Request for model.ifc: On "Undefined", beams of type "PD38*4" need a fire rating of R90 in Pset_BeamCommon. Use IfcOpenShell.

First a look at what the model holds.

```python
import ifcopenshell
import ifcopenshell.util.element

model = ifcopenshell.open("model.ifc")
print(model.schema)
storey = next(s for s in model.by_type("IfcBuildingStorey") if s.Name == "Undefined")
beams = [e for e in ifcopenshell.util.element.get_decomposition(storey) if e.is_a("IfcBeam")]
seen = {}
for e in beams:
    element_type = ifcopenshell.util.element.get_type(e)
    key = (element_type.Name if element_type != e and element_type else None, ifcopenshell.util.element.get_pset(e, "Pset_BeamCommon", "FireRating"))
    seen[key] = seen.get(key, 0) + 1
for (name, value), count in sorted(seen.items(), key=str):
    print(count, "x", name, "|", value)
```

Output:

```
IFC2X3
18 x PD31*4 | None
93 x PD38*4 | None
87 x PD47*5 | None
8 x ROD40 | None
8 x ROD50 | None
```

```python
import ifcopenshell
import ifcopenshell.api.pset
import ifcopenshell.util.element

model = ifcopenshell.open("model.ifc")

storey = next(s for s in model.by_type("IfcBuildingStorey") if s.Name == "Undefined")
beams = [e for e in ifcopenshell.util.element.get_decomposition(storey) if e.is_a("IfcBeam")]

count = 0
for e in beams:
    element_type = ifcopenshell.util.element.get_type(e)
    if element_type in (None, e) or element_type.Name != "PD38*4":
        continue
    found = ifcopenshell.util.element.get_pset(e, "Pset_BeamCommon", should_inherit=False)
    if found:
        pset = model.by_id(found["id"])
        if len(ifcopenshell.util.element.get_elements_by_pset(pset)) > 1:
            pset = ifcopenshell.api.pset.unshare_pset(model, products=[e], pset=pset)[0]
    else:
        pset = ifcopenshell.api.pset.add_pset(model, product=e, name="Pset_BeamCommon")
    ifcopenshell.api.pset.edit_pset(model, pset=pset, properties={"FireRating": "R90"})
    count += 1

print(count, "beams updated")

model.write("model-out.ifc")
```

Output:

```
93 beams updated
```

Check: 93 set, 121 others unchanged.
